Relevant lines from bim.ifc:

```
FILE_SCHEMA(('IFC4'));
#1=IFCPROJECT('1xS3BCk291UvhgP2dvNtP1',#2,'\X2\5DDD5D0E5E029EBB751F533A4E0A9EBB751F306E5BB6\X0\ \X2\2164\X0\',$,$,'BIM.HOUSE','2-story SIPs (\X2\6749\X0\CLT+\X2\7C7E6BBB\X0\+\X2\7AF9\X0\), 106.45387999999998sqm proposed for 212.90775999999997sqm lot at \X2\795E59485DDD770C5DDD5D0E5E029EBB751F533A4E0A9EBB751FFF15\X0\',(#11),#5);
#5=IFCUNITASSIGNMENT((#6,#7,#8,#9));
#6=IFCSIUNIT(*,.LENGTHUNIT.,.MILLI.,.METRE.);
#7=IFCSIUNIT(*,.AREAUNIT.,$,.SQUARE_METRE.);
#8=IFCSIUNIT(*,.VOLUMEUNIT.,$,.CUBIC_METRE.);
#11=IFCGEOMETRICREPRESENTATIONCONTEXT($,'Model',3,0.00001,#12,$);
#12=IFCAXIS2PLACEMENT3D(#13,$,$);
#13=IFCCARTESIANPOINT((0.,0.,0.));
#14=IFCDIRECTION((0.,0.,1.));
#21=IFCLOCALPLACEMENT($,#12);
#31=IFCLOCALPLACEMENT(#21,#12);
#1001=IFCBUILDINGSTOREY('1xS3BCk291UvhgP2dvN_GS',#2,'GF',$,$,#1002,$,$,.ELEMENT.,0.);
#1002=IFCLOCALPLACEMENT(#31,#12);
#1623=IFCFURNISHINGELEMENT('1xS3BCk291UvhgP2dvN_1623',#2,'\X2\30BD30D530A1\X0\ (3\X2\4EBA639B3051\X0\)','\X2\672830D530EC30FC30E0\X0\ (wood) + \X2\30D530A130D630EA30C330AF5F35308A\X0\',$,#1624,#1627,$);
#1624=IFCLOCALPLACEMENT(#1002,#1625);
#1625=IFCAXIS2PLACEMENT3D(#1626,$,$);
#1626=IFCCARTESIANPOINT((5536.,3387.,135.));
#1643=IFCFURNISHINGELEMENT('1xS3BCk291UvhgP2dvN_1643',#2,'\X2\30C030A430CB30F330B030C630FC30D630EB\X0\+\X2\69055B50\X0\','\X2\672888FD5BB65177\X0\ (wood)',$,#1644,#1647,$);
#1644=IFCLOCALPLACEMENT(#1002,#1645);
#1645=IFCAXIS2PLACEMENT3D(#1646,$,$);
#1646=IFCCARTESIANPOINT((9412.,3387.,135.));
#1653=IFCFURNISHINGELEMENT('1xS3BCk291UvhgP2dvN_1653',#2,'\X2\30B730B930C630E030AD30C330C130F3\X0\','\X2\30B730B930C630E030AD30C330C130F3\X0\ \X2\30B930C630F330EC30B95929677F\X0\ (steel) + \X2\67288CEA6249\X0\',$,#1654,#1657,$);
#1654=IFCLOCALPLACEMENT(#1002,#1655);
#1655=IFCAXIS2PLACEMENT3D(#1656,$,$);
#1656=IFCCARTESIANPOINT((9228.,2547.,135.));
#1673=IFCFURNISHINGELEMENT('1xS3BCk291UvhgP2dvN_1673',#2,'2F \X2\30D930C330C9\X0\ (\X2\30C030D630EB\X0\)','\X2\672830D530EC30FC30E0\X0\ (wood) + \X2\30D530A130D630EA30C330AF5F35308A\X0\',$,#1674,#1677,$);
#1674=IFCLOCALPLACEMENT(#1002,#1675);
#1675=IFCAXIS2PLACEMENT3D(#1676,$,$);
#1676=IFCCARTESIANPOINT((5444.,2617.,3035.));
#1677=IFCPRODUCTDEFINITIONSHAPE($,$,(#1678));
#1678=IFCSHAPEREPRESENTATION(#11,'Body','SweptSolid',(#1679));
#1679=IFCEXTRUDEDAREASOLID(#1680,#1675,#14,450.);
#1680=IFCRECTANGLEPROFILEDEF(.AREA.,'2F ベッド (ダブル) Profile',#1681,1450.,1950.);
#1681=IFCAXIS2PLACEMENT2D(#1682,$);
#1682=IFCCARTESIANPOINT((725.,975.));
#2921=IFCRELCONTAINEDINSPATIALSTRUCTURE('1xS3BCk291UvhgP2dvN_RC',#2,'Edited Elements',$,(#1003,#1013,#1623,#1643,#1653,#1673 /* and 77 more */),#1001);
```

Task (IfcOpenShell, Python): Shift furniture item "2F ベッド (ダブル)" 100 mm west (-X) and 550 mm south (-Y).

```python
import ifcopenshell
import ifcopenshell.api.geometry
import ifcopenshell.util.placement
import ifcopenshell.util.unit

model = ifcopenshell.open("bim.ifc")
unit_scale = ifcopenshell.util.unit.calculate_unit_scale(model)

item = model.by_id(1673)
matrix = ifcopenshell.util.placement.get_local_placement(item.ObjectPlacement)
matrix[0, 3] -= 0.1 / unit_scale
matrix[1, 3] -= 0.55 / unit_scale
ifcopenshell.api.geometry.edit_object_placement(model, product=item, matrix=matrix, is_si=False)

print(ifcopenshell.util.placement.get_local_placement(item.ObjectPlacement).round(3) + 0.0)

model.write("bim_edited.ifc")
```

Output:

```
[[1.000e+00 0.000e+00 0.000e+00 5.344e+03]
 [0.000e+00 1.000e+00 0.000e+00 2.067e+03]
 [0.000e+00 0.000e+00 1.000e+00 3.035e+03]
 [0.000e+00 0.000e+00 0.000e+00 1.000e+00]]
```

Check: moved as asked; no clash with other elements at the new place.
